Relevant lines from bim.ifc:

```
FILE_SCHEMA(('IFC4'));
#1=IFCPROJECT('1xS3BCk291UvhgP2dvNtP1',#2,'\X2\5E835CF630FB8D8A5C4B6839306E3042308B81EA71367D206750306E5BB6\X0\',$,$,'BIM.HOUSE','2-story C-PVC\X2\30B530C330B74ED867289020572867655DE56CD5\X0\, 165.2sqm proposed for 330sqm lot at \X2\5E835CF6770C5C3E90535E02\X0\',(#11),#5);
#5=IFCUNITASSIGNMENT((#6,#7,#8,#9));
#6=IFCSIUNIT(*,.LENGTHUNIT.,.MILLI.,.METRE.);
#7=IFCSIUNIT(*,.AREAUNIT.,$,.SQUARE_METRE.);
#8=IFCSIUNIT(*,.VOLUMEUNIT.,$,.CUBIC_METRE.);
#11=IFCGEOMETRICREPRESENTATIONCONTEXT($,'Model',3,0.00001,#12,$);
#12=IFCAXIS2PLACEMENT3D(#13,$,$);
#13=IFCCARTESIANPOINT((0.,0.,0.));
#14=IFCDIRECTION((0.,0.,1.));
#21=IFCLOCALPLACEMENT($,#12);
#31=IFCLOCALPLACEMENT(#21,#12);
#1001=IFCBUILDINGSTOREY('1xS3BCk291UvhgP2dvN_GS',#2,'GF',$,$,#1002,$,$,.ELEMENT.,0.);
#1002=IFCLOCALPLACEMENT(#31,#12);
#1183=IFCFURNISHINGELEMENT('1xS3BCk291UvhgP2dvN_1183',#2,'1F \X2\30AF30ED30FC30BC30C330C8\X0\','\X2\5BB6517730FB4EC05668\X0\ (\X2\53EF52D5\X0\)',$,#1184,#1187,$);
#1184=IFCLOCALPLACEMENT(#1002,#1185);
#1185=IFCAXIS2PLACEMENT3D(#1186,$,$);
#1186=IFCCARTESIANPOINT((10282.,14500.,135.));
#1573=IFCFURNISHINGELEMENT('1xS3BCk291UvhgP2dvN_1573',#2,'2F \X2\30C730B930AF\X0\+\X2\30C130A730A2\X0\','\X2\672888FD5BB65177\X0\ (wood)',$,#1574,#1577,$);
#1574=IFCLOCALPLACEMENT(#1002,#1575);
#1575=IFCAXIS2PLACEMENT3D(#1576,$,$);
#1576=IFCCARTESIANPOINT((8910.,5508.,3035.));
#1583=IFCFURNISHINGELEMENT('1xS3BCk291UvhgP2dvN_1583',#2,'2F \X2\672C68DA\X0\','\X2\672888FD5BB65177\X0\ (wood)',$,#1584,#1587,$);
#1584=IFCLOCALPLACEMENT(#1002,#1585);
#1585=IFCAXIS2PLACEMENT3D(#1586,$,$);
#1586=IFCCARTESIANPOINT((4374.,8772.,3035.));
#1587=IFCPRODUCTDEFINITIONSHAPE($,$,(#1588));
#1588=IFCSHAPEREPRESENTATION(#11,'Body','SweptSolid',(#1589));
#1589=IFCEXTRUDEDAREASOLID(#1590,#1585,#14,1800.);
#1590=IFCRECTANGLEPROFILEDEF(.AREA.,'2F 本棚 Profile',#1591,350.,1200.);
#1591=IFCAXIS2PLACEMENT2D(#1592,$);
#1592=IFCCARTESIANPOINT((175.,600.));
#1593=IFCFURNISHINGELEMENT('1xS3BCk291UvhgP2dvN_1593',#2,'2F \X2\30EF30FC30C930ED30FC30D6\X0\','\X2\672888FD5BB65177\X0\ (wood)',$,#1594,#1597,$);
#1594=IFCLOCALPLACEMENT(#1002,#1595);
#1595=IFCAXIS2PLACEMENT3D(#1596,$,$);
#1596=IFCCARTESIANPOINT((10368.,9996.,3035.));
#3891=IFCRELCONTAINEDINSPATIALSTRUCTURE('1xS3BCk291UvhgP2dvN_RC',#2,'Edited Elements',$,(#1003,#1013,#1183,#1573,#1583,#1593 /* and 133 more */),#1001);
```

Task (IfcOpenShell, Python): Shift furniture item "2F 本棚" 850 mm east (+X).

```python
import ifcopenshell
import ifcopenshell.api.geometry
import ifcopenshell.util.placement

model = ifcopenshell.open("bim.ifc")

item = model.by_guid("1xS3BCk291UvhgP2dvN_1583")
matrix = ifcopenshell.util.placement.get_local_placement(item.ObjectPlacement)
matrix[0, 3] += 850.0
ifcopenshell.api.geometry.edit_object_placement(model, product=item, matrix=matrix, is_si=False)

print(ifcopenshell.util.placement.get_local_placement(item.ObjectPlacement).round(3) + 0.0)

model.write("bim_updated.ifc")
```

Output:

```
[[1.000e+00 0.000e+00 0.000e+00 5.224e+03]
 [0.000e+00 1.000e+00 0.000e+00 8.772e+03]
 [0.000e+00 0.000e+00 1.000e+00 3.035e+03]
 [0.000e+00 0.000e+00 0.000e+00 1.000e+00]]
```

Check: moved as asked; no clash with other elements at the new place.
